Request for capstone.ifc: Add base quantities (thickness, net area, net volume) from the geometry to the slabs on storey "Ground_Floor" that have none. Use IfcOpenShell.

First a look at what the model holds.

```python
import ifcopenshell
import ifcopenshell.util.element
import ifcopenshell.util.unit

model = ifcopenshell.open("capstone.ifc")
print(model.schema)
for unit_type in ("LENGTHUNIT", "AREAUNIT", "VOLUMEUNIT"):
    print(unit_type, ifcopenshell.util.unit.calculate_unit_scale(model, unit_type))
storey = next(s for s in model.by_type("IfcBuildingStorey") if s.Name == "Ground_Floor")
slabs = [e for e in ifcopenshell.util.element.get_decomposition(storey) if e.is_a("IfcSlab")]
for e in sorted(slabs, key=lambda e: e.id()):
    print(e.id(), e.is_a(), e.Name, list(ifcopenshell.util.element.get_psets(e, qtos_only=True)), sep=" | ")
```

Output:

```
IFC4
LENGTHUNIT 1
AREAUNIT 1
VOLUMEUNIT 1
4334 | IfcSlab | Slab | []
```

```python
import ifcopenshell
import ifcopenshell.api.pset
import ifcopenshell.geom
import ifcopenshell.util.element
import ifcopenshell.util.shape
import ifcopenshell.util.unit

model = ifcopenshell.open("capstone.ifc")
unit_scale = ifcopenshell.util.unit.calculate_unit_scale(model)
area_scale = ifcopenshell.util.unit.calculate_unit_scale(model, "AREAUNIT")
volume_scale = ifcopenshell.util.unit.calculate_unit_scale(model, "VOLUMEUNIT")
settings = ifcopenshell.geom.settings()

storey = next(s for s in model.by_type("IfcBuildingStorey") if s.Name == "Ground_Floor")
slabs = [e for e in ifcopenshell.util.element.get_decomposition(storey) if e.is_a("IfcSlab")]

for e in sorted(slabs, key=lambda e: e.id()):
    if ifcopenshell.util.element.get_psets(e, qtos_only=True, should_inherit=False):
        continue
    # Geometry comes back in metres, in the element's own axes.
    shape = ifcopenshell.geom.create_shape(settings, e)
    values = {
        "Width": ifcopenshell.util.shape.get_z(shape.geometry) / unit_scale,
        "NetArea": ifcopenshell.util.shape.get_footprint_area(shape.geometry) / area_scale,
        "NetVolume": ifcopenshell.util.shape.get_volume(shape.geometry) / volume_scale,
    }
    qto = ifcopenshell.api.pset.add_qto(model, product=e, name="Qto_SlabBaseQuantities")
    ifcopenshell.api.pset.edit_qto(model, qto=qto, properties=values)
    print(e.id(), {k: round(v, 3) for k, v in values.items()})

model.write("capstone-out.ifc")
```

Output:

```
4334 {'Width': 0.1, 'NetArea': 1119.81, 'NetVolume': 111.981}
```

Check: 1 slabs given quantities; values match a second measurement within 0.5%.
